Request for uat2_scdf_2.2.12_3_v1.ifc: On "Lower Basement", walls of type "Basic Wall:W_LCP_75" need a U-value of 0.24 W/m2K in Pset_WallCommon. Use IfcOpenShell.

First a look at what the model holds.

```python
import ifcopenshell
import ifcopenshell.util.element

model = ifcopenshell.open("uat2_scdf_2.2.12_3_v1.ifc")
print(model.schema)
storey = next(s for s in model.by_type("IfcBuildingStorey") if s.Name == "Lower Basement")
walls = [e for e in ifcopenshell.util.element.get_decomposition(storey) if e.is_a("IfcWall")]
seen = {}
for e in walls:
    element_type = ifcopenshell.util.element.get_type(e)
    key = (element_type.Name if element_type != e and element_type else None, ifcopenshell.util.element.get_pset(e, "Pset_WallCommon", "ThermalTransmittance"))
    seen[key] = seen.get(key, 0) + 1
for (name, value), count in sorted(seen.items(), key=str):
    print(count, "x", name, "|", value)
```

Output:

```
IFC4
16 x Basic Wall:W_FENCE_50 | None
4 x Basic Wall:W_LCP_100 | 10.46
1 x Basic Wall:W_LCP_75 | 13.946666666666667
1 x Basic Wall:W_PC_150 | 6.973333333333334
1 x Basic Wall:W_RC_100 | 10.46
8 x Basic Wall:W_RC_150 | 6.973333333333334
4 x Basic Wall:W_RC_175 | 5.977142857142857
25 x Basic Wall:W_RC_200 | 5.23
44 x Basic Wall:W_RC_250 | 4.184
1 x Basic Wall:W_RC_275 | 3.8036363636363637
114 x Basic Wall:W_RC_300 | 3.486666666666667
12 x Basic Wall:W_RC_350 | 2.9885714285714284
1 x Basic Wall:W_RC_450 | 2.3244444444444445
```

```python
import ifcopenshell
import ifcopenshell.api.pset
import ifcopenshell.util.element

model = ifcopenshell.open("uat2_scdf_2.2.12_3_v1.ifc")

storey = next(s for s in model.by_type("IfcBuildingStorey") if s.Name == "Lower Basement")
walls = [e for e in ifcopenshell.util.element.get_decomposition(storey) if e.is_a("IfcWall")]

count = 0
for e in walls:
    element_type = ifcopenshell.util.element.get_type(e)
    if element_type in (None, e) or element_type.Name != "Basic Wall:W_LCP_75":
        continue
    # add_pset returns the element's existing set when there is one.
    pset = ifcopenshell.api.pset.add_pset(model, product=e, name="Pset_WallCommon")
    ifcopenshell.api.pset.edit_pset(model, pset=pset, properties={"ThermalTransmittance": 0.24})
    count += 1

print(count, "walls updated")

model.write("uat2_scdf_2.2.12_3_v1-out.ifc")
```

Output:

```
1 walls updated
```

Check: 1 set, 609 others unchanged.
